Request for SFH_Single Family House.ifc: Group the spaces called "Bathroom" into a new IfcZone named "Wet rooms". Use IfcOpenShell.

First a look at what the model holds.

```python
import ifcopenshell

model = ifcopenshell.open("SFH_Single Family House.ifc")
print(model.schema)
seen = {}
for space in model.by_type("IfcSpace"):
    seen[space.LongName] = seen.get(space.LongName, 0) + 1
for name, count in sorted(seen.items(), key=str):
    print(count, "x", name)
print("zones:", [z.Name for z in model.by_type("IfcZone")][:20])
```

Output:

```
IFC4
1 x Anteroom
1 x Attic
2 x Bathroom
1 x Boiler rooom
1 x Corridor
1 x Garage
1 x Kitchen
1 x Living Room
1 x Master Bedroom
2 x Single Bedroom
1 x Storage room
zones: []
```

```python
import ifcopenshell
import ifcopenshell.api.group
import ifcopenshell.api.root

model = ifcopenshell.open("SFH_Single Family House.ifc")

names = {"Bathroom"}
spaces = [s for s in model.by_type("IfcSpace") if s.LongName in names]

zone = ifcopenshell.api.root.create_entity(model, ifc_class="IfcZone", name="Wet rooms")
ifcopenshell.api.group.assign_group(model, products=spaces, group=zone)
print(len(spaces), "spaces in", zone.Name)

model.write("SFH_Single Family House-out.ifc")
```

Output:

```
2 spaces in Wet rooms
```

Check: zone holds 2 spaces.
